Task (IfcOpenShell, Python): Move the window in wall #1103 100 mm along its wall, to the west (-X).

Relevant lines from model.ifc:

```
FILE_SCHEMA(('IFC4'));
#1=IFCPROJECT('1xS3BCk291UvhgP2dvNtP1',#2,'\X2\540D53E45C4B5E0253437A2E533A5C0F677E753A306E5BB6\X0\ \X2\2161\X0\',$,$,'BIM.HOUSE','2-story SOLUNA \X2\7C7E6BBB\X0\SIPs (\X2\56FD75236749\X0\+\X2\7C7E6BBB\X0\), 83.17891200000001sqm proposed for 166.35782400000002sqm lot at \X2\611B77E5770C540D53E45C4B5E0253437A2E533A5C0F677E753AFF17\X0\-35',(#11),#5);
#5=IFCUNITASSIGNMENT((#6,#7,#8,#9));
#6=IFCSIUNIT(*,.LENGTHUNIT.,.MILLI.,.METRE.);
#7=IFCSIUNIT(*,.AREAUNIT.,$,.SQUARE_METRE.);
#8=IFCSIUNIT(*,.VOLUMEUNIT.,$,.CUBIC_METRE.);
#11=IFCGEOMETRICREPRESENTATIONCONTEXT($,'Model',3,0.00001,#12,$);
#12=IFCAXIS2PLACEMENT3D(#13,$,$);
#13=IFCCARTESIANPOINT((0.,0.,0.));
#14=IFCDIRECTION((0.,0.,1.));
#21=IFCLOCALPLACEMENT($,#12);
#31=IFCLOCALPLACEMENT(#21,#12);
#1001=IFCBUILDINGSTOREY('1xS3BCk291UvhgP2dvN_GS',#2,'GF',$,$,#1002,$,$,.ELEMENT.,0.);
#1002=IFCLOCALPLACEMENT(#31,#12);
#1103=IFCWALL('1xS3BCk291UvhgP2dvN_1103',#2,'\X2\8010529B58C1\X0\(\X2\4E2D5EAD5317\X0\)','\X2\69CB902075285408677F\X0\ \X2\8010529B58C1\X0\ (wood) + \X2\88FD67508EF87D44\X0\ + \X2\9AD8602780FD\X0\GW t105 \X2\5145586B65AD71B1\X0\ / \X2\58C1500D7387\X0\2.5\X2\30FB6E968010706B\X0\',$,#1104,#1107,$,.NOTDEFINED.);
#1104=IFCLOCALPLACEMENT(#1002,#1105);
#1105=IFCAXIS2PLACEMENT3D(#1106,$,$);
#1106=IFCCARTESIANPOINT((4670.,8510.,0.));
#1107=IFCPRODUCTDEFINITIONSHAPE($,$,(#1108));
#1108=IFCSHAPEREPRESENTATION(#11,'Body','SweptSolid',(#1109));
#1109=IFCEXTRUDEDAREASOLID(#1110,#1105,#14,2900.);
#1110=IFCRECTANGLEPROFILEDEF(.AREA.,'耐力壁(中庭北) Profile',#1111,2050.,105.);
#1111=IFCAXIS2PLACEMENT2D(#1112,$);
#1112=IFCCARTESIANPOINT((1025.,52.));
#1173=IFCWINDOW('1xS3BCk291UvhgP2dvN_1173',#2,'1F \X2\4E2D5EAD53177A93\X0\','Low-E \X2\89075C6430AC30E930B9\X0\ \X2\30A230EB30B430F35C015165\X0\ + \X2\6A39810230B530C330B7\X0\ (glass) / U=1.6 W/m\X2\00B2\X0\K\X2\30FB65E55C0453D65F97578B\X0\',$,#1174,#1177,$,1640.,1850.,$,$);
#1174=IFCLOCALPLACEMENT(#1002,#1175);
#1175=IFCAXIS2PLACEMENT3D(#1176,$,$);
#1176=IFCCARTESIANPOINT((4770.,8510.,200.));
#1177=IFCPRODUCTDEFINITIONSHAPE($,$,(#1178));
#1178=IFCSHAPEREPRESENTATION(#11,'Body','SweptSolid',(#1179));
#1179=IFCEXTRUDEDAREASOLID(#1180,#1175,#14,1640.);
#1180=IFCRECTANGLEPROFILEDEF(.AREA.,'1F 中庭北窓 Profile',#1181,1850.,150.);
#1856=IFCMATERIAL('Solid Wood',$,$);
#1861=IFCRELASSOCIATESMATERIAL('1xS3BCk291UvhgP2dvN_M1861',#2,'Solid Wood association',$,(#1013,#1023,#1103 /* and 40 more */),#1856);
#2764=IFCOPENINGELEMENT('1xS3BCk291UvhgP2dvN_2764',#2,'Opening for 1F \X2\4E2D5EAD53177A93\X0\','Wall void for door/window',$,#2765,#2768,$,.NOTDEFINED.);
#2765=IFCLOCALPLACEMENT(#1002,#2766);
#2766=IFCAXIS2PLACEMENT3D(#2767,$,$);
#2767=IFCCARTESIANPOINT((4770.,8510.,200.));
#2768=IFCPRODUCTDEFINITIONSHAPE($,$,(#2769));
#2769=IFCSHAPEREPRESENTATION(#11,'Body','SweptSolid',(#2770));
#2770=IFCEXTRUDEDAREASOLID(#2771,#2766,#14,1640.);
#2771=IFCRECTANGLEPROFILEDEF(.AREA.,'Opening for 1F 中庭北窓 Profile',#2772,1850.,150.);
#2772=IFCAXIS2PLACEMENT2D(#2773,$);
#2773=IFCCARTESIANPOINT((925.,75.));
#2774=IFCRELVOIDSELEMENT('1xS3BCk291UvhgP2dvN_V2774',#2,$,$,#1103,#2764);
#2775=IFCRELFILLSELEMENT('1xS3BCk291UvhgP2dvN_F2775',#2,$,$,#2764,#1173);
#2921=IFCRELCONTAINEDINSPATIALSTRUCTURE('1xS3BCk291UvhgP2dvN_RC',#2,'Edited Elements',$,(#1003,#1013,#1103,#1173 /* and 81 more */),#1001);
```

```python
import ifcopenshell
import ifcopenshell.api.geometry
import ifcopenshell.util.placement

model = ifcopenshell.open("model.ifc")

window = model.by_guid("1xS3BCk291UvhgP2dvN_1173")
opening = window.FillsVoids[0].RelatingOpeningElement
wall = opening.VoidsElements[0].RelatingBuildingElement

wall_matrix = ifcopenshell.util.placement.get_local_placement(wall.ObjectPlacement)
shift = wall_matrix[:3, 0] * -100.0
before = ifcopenshell.util.placement.get_local_placement(window.ObjectPlacement)[:3, 3].copy()

# The window is not placed relative to its opening, so move both.
for product in (opening, window):
    matrix = ifcopenshell.util.placement.get_local_placement(product.ObjectPlacement)
    matrix[:3, 3] += shift
    ifcopenshell.api.geometry.edit_object_placement(model, product=product, matrix=matrix, is_si=False)

after = ifcopenshell.util.placement.get_local_placement(window.ObjectPlacement)[:3, 3]
print("window moved by", (after - before).round(3) + 0.0)

model.write("model_edited.ifc")
```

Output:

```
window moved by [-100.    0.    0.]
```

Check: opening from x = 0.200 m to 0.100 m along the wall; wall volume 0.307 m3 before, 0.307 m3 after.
